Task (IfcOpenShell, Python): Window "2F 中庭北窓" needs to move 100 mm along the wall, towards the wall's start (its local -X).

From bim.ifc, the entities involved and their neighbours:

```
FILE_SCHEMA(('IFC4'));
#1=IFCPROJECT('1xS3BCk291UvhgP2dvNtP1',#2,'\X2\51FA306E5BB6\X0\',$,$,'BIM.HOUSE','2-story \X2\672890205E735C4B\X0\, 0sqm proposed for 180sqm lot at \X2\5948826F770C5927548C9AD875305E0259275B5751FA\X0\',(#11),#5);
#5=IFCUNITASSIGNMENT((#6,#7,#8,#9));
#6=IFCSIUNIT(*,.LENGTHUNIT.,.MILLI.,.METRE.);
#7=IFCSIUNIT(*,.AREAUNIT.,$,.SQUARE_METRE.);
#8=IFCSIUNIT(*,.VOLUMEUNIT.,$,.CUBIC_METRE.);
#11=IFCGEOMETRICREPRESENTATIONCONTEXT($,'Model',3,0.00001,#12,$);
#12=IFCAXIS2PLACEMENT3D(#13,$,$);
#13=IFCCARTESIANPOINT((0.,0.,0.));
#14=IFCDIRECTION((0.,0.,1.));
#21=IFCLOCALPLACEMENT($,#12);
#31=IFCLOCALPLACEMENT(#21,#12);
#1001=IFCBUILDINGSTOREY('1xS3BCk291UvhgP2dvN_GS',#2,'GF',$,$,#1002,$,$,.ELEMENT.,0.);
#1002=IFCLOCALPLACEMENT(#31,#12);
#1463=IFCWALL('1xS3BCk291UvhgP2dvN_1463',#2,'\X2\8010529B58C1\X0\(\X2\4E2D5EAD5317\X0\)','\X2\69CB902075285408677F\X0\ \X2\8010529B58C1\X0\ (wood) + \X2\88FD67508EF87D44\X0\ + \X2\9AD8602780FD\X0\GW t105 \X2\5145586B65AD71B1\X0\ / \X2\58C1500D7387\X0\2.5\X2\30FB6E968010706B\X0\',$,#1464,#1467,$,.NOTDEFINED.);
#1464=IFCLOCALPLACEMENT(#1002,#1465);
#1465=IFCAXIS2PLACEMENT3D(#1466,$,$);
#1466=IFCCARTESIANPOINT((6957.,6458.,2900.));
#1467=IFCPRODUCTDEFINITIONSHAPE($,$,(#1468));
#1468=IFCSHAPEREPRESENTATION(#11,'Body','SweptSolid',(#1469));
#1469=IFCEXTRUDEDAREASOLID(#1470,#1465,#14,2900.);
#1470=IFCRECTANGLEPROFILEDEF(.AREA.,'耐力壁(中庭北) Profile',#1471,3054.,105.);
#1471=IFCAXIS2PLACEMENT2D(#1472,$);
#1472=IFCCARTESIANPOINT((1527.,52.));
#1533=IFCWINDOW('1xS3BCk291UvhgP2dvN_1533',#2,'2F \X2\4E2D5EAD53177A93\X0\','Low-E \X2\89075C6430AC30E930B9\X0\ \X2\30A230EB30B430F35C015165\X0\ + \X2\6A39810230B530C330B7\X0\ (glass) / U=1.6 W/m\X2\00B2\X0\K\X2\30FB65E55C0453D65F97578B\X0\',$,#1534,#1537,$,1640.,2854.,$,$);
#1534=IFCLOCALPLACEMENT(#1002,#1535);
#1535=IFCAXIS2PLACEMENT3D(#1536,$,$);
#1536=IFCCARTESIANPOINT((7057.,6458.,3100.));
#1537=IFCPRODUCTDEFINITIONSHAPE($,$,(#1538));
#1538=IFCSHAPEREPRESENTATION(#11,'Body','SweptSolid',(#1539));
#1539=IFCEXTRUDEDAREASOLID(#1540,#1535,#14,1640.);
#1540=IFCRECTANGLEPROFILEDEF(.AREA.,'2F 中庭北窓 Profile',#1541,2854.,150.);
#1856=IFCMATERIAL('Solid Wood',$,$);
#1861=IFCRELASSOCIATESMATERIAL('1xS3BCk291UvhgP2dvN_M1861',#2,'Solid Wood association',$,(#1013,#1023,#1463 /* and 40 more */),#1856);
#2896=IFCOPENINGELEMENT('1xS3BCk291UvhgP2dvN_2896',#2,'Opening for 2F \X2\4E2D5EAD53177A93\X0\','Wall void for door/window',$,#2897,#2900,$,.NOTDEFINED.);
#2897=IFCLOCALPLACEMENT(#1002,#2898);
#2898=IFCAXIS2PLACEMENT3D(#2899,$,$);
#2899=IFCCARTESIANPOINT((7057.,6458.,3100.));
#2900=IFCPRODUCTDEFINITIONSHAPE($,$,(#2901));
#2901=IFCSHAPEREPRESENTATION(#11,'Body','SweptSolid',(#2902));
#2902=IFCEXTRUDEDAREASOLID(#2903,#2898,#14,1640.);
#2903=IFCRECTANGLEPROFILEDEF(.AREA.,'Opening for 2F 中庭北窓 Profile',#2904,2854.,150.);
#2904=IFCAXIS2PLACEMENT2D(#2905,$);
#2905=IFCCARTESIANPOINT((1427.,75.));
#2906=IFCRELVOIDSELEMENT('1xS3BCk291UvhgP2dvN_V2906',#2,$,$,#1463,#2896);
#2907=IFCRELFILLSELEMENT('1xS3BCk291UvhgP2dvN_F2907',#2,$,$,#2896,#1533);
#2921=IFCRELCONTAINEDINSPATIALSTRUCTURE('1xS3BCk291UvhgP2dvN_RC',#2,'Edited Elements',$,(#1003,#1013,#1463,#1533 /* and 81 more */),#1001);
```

```python
import ifcopenshell
import ifcopenshell.api.geometry
import ifcopenshell.util.placement

model = ifcopenshell.open("bim.ifc")

window = model.by_guid("1xS3BCk291UvhgP2dvN_1533")
opening = window.FillsVoids[0].RelatingOpeningElement
wall = opening.VoidsElements[0].RelatingBuildingElement

wall_matrix = ifcopenshell.util.placement.get_local_placement(wall.ObjectPlacement)
shift = wall_matrix[:3, 0] * -100.0
before = ifcopenshell.util.placement.get_local_placement(window.ObjectPlacement)[:3, 3].copy()

# The window is not placed relative to its opening, so move both.
for product in (opening, window):
    matrix = ifcopenshell.util.placement.get_local_placement(product.ObjectPlacement)
    matrix[:3, 3] += shift
    ifcopenshell.api.geometry.edit_object_placement(model, product=product, matrix=matrix, is_si=False)

after = ifcopenshell.util.placement.get_local_placement(window.ObjectPlacement)[:3, 3]
print("window moved by", (after - before).round(3) + 0.0)

model.write("bim_v2.ifc")
```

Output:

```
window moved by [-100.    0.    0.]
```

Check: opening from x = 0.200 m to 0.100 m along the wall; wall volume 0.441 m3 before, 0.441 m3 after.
